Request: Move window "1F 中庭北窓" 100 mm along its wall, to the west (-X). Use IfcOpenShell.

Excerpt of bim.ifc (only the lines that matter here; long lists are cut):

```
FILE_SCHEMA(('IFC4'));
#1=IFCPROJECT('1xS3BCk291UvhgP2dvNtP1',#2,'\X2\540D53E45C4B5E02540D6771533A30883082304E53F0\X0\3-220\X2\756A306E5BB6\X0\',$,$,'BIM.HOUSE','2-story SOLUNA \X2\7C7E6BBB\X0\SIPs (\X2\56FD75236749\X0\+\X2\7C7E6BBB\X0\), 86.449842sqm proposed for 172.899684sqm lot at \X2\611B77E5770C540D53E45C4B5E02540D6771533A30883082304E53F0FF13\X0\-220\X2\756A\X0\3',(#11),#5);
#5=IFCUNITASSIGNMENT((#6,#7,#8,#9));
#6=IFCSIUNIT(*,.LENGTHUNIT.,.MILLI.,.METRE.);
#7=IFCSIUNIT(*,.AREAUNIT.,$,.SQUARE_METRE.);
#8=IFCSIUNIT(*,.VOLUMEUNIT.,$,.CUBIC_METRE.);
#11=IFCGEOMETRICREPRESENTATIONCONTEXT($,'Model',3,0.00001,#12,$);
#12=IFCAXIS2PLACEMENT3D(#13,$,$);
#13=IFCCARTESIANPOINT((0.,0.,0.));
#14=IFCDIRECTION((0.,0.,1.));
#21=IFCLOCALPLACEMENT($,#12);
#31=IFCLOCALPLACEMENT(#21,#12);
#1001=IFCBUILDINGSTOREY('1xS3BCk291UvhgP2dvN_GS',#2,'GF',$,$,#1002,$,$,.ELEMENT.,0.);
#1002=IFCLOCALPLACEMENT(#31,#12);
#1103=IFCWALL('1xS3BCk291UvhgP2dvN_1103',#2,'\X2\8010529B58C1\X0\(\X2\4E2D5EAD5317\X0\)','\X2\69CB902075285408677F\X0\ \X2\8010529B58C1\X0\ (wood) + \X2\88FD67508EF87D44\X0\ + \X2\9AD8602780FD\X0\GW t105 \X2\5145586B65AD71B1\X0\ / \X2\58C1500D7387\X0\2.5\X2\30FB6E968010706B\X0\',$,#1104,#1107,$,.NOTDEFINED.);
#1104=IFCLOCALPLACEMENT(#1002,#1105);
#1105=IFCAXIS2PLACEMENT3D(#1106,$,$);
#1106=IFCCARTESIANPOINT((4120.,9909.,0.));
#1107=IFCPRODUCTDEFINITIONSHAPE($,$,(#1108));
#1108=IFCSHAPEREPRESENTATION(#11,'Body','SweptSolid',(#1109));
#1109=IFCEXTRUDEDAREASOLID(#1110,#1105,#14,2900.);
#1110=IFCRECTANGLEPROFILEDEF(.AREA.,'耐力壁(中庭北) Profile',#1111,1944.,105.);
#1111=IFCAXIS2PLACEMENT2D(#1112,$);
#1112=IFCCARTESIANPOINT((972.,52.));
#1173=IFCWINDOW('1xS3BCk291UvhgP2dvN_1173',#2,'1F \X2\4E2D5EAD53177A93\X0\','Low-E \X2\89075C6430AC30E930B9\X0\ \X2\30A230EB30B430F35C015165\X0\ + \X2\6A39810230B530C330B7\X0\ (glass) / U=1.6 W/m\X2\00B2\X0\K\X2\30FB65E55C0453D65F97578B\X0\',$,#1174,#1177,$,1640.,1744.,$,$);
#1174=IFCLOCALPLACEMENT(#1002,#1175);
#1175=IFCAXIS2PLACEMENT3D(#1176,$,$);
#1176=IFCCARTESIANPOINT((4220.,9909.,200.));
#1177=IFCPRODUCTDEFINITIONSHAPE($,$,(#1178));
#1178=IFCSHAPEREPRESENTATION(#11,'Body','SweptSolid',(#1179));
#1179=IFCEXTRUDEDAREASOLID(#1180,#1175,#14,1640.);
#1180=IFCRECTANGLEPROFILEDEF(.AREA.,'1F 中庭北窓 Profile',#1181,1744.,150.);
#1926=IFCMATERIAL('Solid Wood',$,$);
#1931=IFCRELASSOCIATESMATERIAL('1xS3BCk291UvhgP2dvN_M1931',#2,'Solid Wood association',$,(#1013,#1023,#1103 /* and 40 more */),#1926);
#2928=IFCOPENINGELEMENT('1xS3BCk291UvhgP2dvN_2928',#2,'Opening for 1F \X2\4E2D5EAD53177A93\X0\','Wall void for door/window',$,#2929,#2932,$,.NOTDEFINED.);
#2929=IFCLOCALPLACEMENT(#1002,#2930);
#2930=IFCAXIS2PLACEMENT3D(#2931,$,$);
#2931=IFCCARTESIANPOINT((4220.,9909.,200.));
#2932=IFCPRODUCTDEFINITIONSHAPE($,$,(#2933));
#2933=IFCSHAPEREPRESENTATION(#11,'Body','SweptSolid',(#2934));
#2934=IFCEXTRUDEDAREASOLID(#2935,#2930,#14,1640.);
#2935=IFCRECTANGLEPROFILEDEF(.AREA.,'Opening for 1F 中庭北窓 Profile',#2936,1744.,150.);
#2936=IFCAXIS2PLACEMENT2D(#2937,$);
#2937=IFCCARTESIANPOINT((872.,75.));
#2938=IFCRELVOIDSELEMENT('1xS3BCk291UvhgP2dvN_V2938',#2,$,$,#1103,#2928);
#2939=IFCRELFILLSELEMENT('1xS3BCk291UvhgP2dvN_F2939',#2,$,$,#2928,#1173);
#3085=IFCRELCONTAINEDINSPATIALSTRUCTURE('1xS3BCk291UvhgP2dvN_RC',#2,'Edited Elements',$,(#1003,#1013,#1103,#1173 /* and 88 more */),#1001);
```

```python
import ifcopenshell
import ifcopenshell.api.geometry
import ifcopenshell.util.placement
import ifcopenshell.util.unit

model = ifcopenshell.open("bim.ifc")
unit_scale = ifcopenshell.util.unit.calculate_unit_scale(model)

window = model.by_id(1173)
opening = window.FillsVoids[0].RelatingOpeningElement
wall = opening.VoidsElements[0].RelatingBuildingElement

wall_matrix = ifcopenshell.util.placement.get_local_placement(wall.ObjectPlacement)
shift = wall_matrix[:3, 0] * -0.1 / unit_scale
before = ifcopenshell.util.placement.get_local_placement(window.ObjectPlacement)[:3, 3].copy()

# The window is not placed relative to its opening, so move both.
for product in (opening, window):
    matrix = ifcopenshell.util.placement.get_local_placement(product.ObjectPlacement)
    matrix[:3, 3] += shift
    ifcopenshell.api.geometry.edit_object_placement(model, product=product, matrix=matrix, is_si=False)

after = ifcopenshell.util.placement.get_local_placement(window.ObjectPlacement)[:3, 3]
print("window moved by", (after - before).round(3) + 0.0)

model.write("bim_edited.ifc")
```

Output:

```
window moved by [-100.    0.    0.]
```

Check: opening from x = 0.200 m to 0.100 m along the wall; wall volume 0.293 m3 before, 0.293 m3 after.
